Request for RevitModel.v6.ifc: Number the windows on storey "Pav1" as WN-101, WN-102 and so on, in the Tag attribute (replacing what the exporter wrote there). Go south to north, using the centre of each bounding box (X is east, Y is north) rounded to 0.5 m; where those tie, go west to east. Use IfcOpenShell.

First a look at what the model holds.

```python
import ifcopenshell
import ifcopenshell.util.element
import ifcopenshell.util.placement

model = ifcopenshell.open("RevitModel.v6.ifc")
print(model.schema)
storey = next(s for s in model.by_type("IfcBuildingStorey") if s.Name == "Pav1")
windows = [e for e in ifcopenshell.util.element.get_decomposition(storey) if e.is_a("IfcWindow")]
for e in sorted(windows, key=lambda e: e.id()):
    origin = ifcopenshell.util.placement.get_local_placement(e.ObjectPlacement)[:3, 3]
    print(e.id(), e.Tag, e.Name, origin.round(2) + 0.0, sep=" | ")
```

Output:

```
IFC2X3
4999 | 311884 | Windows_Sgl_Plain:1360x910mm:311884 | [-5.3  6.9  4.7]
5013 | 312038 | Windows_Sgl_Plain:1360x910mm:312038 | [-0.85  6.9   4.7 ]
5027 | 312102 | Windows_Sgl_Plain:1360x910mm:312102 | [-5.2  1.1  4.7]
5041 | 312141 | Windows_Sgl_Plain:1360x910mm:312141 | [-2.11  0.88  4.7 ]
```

```python
import ifcopenshell
import ifcopenshell.geom
import ifcopenshell.util.element
import ifcopenshell.util.shape

model = ifcopenshell.open("RevitModel.v6.ifc")
settings = ifcopenshell.geom.settings()
settings.set("use-world-coords", True)


def centre(element):
    shape = ifcopenshell.geom.create_shape(settings, element)
    return ifcopenshell.util.shape.get_bbox_centroid(shape.geometry)


storey = next(s for s in model.by_type("IfcBuildingStorey") if s.Name == "Pav1")
windows = [e for e in ifcopenshell.util.element.get_decomposition(storey) if e.is_a("IfcWindow")]

# Insertion points can sit at a corner or the storey origin, so sort by the geometry (in metres).
centres = {e: centre(e) for e in windows}
windows.sort(key=lambda e: (round(centres[e][1] / 0.5), centres[e][0]))

for i, e in enumerate(windows, start=1):
    number = f"WN-1{i:02d}"
    e.Tag = number
    print(e.id(), number)

model.write("RevitModel.v6_edited.ifc")
```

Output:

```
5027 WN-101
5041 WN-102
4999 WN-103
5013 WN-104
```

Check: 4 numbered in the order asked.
